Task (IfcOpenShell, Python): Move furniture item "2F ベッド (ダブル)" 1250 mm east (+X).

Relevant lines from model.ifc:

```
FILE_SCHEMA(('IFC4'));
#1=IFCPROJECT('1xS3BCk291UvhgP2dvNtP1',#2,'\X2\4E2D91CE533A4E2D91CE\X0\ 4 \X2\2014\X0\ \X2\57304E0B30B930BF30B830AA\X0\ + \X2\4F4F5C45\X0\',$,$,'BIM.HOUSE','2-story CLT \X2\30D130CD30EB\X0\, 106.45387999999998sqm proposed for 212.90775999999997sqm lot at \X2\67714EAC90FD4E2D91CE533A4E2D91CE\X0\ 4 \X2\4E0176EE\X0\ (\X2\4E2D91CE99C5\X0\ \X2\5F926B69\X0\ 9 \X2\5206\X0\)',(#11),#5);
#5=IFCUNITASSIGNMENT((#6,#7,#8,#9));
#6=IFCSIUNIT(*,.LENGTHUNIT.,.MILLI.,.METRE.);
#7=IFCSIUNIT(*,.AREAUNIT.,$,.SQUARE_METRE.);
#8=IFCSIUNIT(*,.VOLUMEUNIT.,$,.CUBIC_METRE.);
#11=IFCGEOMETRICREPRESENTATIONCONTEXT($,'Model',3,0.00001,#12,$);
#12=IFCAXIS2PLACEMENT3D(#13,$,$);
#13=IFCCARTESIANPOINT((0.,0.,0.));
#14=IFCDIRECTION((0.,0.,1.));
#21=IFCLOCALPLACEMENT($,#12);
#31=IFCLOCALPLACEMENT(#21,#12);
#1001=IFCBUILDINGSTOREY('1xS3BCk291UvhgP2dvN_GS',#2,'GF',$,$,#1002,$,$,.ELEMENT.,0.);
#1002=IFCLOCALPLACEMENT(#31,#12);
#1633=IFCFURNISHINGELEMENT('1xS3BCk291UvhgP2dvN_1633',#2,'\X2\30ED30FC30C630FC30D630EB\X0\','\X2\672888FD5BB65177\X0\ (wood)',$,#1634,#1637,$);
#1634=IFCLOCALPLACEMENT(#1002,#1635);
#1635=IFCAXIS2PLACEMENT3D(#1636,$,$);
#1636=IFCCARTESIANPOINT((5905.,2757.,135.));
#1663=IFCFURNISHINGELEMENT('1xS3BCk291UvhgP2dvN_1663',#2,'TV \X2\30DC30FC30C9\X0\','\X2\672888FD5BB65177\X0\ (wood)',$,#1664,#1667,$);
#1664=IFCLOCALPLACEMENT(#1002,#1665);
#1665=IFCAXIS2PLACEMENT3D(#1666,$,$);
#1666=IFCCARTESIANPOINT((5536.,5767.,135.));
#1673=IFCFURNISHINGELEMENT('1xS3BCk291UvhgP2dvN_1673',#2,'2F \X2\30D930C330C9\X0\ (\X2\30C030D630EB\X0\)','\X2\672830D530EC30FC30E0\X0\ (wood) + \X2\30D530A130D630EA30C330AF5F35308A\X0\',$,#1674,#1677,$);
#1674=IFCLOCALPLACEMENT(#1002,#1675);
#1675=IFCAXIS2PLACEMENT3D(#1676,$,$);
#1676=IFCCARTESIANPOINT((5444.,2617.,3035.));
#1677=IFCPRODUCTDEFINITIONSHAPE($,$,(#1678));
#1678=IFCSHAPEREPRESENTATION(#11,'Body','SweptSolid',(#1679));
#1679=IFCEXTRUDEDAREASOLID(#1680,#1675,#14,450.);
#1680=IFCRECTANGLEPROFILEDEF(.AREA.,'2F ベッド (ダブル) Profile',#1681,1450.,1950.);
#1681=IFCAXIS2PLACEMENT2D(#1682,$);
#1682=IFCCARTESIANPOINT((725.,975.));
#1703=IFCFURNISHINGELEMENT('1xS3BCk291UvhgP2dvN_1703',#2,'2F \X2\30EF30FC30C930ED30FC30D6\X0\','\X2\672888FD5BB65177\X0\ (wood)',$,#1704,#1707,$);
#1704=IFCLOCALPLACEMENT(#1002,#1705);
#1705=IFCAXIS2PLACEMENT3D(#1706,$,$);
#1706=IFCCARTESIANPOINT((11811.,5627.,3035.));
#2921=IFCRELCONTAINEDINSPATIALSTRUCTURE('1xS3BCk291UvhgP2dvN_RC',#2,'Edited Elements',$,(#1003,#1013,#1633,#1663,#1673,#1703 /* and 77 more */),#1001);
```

```python
import ifcopenshell
import ifcopenshell.api.geometry
import ifcopenshell.util.placement
import ifcopenshell.util.unit

model = ifcopenshell.open("model.ifc")
unit_scale = ifcopenshell.util.unit.calculate_unit_scale(model)

item = model.by_guid("1xS3BCk291UvhgP2dvN_1673")
matrix = ifcopenshell.util.placement.get_local_placement(item.ObjectPlacement)
matrix[0, 3] += 1.25 / unit_scale
ifcopenshell.api.geometry.edit_object_placement(model, product=item, matrix=matrix, is_si=False)

print(ifcopenshell.util.placement.get_local_placement(item.ObjectPlacement).round(3) + 0.0)

model.write("model_rev.ifc")
```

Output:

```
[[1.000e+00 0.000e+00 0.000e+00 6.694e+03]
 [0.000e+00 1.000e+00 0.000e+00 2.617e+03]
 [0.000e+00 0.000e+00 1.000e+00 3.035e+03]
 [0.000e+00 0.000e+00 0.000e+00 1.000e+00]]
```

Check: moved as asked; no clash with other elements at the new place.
